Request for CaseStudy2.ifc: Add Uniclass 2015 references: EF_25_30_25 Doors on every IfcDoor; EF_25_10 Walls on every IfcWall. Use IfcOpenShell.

First a look at what the model holds.

```python
import ifcopenshell

model = ifcopenshell.open("CaseStudy2.ifc")
print(model.schema)
print("classifications:", [c.Name for c in model.by_type("IfcClassification")])
for ifc_class in ("IfcDoor", "IfcRoof", "IfcStair", "IfcWall", "IfcWindow"):
    print(ifc_class, len(model.by_type(ifc_class)))
```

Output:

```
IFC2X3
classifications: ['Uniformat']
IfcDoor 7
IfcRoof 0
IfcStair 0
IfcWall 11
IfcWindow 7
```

```python
import ifcopenshell
import ifcopenshell.api.classification

model = ifcopenshell.open("CaseStudy2.ifc")

# IFC2X3 requires Source and Edition and has no link from the project to the system.
system = model.create_entity("IfcClassification", Source="NBS", Edition="2015", Name="Uniclass 2015")

codes = {
    "IfcDoor": ("EF_25_30_25", "Doors"),
    "IfcWall": ("EF_25_10", "Walls"),
}
for ifc_class, (code, name) in codes.items():
    products = model.by_type(ifc_class)
    ifcopenshell.api.classification.add_reference(
        model, products=products, classification=system, identification=code, name=name
    )
    print(code, len(products))

model.write("CaseStudy2-out.ifc")
```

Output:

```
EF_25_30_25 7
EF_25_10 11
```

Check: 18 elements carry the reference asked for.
